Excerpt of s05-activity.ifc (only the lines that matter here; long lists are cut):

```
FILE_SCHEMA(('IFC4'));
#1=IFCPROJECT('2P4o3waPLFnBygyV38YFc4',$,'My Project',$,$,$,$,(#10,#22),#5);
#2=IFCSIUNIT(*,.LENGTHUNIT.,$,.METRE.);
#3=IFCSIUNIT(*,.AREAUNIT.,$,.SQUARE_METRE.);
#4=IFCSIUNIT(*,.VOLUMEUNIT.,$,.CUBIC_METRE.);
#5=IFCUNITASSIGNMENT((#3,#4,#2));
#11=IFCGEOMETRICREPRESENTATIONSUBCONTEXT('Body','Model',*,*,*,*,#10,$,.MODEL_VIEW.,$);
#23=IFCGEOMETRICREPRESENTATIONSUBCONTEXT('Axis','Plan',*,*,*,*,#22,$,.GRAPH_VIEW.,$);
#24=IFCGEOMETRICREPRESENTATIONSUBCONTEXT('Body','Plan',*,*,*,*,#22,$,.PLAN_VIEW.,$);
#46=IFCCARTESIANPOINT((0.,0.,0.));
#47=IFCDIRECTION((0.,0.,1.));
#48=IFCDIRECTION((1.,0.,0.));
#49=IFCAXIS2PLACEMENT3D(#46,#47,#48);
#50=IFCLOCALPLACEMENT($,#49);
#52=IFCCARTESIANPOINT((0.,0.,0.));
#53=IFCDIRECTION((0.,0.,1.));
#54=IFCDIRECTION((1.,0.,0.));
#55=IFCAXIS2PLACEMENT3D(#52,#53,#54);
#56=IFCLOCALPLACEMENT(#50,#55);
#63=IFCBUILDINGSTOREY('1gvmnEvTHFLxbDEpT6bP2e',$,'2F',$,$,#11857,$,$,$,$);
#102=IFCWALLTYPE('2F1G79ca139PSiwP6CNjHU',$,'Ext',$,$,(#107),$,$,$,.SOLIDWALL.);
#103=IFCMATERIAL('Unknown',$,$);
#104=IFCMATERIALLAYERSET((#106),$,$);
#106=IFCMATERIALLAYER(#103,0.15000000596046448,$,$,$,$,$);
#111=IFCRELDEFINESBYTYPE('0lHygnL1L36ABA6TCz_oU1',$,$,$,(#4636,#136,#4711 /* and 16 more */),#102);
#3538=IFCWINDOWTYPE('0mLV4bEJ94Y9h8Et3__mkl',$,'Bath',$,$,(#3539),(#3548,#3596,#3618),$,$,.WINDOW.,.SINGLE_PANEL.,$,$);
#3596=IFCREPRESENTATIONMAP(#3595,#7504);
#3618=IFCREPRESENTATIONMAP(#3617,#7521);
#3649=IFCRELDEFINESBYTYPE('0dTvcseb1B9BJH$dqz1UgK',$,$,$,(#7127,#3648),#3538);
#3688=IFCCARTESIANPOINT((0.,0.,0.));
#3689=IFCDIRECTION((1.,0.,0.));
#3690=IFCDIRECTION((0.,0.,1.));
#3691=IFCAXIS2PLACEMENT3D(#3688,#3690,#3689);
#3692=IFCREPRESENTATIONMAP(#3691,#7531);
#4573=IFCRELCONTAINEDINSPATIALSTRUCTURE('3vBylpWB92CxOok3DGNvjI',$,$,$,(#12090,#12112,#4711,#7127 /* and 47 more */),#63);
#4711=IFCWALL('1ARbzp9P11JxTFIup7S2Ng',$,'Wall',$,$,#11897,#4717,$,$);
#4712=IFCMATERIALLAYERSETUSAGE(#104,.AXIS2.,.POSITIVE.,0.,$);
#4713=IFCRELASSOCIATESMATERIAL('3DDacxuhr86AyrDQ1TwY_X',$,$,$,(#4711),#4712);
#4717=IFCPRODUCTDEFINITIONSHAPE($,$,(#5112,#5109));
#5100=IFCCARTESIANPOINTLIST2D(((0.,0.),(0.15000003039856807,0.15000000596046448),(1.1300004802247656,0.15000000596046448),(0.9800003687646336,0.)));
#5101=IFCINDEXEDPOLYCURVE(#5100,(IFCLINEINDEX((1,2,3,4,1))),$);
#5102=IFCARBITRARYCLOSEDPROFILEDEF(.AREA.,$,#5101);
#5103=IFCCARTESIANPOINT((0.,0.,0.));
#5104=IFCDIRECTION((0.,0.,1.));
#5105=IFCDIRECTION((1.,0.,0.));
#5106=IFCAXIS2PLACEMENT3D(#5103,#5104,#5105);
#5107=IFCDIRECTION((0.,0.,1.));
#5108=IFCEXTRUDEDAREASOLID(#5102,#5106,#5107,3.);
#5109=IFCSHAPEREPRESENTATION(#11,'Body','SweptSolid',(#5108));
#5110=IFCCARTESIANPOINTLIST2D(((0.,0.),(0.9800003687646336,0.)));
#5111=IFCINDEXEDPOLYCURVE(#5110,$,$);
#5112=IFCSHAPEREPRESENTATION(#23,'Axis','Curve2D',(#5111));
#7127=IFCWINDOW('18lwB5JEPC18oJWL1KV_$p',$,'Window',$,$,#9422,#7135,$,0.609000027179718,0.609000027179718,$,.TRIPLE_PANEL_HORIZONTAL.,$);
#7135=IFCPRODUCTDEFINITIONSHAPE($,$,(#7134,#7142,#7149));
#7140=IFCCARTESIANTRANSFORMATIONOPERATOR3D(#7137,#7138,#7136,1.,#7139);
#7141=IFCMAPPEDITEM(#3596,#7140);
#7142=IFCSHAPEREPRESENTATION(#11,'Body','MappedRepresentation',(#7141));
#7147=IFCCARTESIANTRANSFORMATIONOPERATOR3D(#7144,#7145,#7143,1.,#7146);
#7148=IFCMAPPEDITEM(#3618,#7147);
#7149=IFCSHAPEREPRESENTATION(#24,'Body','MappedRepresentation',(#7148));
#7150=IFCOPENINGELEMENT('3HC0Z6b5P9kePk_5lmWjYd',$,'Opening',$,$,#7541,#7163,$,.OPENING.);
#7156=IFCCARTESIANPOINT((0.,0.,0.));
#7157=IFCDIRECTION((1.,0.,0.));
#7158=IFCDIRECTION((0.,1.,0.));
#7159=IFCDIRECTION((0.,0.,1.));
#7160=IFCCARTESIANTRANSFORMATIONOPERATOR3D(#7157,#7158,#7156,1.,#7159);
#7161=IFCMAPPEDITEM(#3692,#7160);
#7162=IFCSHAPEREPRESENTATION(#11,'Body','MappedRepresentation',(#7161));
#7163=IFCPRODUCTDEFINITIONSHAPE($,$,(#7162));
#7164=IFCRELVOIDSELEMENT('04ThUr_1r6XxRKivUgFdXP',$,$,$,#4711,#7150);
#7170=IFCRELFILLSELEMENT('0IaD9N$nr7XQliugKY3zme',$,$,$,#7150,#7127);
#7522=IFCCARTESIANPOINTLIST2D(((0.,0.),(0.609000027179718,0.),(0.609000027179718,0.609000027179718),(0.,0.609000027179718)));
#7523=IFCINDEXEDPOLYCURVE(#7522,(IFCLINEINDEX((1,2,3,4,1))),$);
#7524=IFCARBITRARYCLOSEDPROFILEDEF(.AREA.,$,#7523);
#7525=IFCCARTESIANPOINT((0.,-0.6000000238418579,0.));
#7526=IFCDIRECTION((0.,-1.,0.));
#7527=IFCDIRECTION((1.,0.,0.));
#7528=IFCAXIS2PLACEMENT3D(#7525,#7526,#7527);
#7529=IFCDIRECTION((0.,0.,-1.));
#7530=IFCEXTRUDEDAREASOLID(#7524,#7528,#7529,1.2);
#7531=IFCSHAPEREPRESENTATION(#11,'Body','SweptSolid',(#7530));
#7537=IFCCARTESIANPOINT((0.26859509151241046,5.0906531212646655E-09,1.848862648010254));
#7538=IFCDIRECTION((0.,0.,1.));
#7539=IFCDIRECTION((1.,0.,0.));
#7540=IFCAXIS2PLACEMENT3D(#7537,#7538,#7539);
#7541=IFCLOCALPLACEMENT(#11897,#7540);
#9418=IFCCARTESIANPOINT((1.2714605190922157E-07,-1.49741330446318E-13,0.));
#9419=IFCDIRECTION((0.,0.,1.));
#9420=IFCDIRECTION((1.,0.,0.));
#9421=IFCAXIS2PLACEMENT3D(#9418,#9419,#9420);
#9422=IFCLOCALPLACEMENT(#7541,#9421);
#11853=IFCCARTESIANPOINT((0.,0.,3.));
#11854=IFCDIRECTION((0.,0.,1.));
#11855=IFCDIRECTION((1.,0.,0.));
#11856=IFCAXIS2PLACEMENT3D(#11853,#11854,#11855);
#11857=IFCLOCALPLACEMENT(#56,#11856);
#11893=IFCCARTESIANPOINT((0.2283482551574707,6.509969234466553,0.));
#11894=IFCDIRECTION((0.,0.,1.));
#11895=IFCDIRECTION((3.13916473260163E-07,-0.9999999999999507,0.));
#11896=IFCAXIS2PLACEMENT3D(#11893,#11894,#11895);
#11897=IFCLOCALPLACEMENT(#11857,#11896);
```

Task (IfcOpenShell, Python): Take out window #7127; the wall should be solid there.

```python
import ifcopenshell
import ifcopenshell.api.feature
import ifcopenshell.api.root
import ifcopenshell.geom
import ifcopenshell.util.shape

model = ifcopenshell.open("s05-activity.ifc")
settings = ifcopenshell.geom.settings()


def volume(element):
    """Net volume in cubic metres, openings subtracted."""
    shape = ifcopenshell.geom.create_shape(settings, element)
    return ifcopenshell.util.shape.get_volume(shape.geometry)


window = model.by_guid("18lwB5JEPC18oJWL1KV_$p")
opening = window.FillsVoids[0].RelatingOpeningElement
wall = opening.VoidsElements[0].RelatingBuildingElement
before = volume(wall)

ifcopenshell.api.root.remove_product(model, product=window)
ifcopenshell.api.feature.remove_feature(model, feature=opening)

after = volume(wall)

print(f"wall volume {before:.3f} -> {after:.3f} m3")

model.write("s05-activity_v2.ifc")
```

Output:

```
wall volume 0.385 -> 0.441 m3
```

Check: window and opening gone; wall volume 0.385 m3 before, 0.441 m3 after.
